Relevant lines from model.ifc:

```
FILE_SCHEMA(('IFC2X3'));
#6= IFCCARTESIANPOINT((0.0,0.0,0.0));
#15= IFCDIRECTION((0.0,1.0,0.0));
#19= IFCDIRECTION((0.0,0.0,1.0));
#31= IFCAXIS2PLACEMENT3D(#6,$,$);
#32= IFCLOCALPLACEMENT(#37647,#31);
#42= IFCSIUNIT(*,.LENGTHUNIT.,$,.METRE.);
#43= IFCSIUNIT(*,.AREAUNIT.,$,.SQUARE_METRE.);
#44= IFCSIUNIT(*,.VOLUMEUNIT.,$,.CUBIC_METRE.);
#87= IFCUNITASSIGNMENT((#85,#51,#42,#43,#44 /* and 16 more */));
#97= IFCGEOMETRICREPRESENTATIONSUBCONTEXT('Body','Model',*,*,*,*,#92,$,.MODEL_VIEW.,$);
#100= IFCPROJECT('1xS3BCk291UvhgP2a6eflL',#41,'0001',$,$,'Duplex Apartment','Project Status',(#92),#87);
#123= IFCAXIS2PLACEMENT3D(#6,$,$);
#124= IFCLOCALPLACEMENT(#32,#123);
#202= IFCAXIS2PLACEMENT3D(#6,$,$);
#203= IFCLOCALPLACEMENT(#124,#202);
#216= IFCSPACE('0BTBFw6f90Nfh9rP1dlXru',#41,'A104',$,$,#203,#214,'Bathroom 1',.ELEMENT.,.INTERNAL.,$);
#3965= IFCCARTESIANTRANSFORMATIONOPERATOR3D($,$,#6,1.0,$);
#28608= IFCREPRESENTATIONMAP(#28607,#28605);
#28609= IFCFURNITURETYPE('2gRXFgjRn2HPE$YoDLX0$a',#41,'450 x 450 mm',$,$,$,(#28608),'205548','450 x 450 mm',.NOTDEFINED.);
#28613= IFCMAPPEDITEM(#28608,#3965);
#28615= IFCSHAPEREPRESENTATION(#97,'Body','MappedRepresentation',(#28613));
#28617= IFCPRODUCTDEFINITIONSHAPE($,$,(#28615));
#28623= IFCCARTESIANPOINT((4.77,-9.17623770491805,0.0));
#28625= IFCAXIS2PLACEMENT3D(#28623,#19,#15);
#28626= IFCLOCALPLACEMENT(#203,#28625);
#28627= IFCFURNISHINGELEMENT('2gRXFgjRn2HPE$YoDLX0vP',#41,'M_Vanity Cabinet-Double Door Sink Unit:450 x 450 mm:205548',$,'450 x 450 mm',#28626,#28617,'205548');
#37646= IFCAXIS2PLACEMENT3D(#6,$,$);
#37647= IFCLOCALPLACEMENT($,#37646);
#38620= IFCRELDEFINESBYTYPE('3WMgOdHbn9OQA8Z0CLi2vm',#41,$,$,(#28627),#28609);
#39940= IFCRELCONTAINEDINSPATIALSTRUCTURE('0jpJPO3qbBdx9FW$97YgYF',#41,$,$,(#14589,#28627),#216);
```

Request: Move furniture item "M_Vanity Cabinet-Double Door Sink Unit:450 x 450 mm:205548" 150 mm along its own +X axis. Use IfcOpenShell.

```python
import ifcopenshell
import ifcopenshell.api.geometry
import ifcopenshell.util.placement
import ifcopenshell.util.unit

model = ifcopenshell.open("model.ifc")
unit_scale = ifcopenshell.util.unit.calculate_unit_scale(model)

item = model.by_guid("2gRXFgjRn2HPE$YoDLX0vP")
matrix = ifcopenshell.util.placement.get_local_placement(item.ObjectPlacement)
matrix[:3, 3] += matrix[:3, 0] * 0.15 / unit_scale
ifcopenshell.api.geometry.edit_object_placement(model, product=item, matrix=matrix, is_si=False)

print(ifcopenshell.util.placement.get_local_placement(item.ObjectPlacement).round(3) + 0.0)

model.write("model_rev.ifc")
```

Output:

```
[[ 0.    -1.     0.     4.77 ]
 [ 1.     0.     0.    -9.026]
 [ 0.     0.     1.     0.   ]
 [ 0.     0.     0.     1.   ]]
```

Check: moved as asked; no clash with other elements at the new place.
